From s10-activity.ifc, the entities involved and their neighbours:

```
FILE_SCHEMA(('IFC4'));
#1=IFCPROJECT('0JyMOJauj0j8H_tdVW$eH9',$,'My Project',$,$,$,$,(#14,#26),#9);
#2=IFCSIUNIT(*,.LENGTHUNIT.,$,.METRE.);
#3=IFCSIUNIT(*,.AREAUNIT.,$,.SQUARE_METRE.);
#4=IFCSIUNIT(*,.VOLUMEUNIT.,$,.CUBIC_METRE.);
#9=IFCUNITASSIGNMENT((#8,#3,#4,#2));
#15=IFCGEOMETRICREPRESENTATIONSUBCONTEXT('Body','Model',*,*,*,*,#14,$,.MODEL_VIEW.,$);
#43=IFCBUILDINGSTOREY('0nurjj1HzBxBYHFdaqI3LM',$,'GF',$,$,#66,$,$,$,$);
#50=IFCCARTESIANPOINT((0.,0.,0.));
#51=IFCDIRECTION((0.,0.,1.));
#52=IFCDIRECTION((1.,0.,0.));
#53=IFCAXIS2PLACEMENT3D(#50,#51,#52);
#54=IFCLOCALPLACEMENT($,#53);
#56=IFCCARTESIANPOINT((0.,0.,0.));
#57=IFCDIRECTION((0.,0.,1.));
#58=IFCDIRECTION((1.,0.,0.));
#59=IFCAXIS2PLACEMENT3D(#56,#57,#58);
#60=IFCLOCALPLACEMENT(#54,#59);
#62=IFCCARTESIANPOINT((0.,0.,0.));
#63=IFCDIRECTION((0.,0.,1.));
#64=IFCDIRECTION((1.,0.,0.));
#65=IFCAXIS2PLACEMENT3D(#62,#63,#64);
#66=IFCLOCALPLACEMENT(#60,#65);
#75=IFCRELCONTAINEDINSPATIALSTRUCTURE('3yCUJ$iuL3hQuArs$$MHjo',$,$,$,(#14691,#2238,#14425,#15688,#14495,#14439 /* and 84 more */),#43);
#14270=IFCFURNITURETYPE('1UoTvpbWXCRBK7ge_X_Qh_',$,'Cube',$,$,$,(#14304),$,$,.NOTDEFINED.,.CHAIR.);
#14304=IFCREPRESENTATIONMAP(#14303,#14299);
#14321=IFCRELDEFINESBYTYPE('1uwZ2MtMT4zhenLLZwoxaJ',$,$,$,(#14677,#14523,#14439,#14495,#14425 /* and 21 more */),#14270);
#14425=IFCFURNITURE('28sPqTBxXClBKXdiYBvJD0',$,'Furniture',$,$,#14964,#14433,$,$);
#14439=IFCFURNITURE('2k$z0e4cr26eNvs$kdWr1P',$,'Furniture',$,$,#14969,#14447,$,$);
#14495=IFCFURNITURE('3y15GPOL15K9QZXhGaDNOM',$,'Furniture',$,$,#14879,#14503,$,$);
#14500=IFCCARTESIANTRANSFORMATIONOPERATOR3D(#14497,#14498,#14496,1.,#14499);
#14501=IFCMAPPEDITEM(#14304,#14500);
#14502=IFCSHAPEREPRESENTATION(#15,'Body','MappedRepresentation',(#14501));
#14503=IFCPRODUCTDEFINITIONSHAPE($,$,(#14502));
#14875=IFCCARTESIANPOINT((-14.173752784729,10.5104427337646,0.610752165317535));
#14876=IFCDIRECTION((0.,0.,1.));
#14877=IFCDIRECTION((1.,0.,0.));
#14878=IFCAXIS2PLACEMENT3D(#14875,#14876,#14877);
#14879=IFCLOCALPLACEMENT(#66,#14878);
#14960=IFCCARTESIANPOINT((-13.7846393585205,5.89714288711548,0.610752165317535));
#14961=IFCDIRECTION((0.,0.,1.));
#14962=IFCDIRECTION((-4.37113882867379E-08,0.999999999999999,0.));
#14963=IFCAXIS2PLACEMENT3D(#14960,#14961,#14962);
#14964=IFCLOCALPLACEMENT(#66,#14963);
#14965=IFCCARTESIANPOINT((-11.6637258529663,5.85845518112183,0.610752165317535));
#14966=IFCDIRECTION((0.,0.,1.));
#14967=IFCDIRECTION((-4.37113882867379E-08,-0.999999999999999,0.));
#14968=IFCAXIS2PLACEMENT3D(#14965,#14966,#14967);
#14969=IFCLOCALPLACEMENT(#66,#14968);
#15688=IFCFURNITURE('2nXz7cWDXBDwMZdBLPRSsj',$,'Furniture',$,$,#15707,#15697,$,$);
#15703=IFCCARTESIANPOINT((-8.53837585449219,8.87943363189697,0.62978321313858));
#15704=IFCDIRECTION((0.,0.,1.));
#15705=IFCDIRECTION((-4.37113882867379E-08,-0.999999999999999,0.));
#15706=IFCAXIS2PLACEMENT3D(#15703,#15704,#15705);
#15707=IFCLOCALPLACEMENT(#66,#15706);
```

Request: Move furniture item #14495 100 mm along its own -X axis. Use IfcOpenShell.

```python
import ifcopenshell
import ifcopenshell.api.geometry
import ifcopenshell.util.placement
import ifcopenshell.util.unit

model = ifcopenshell.open("s10-activity.ifc")
unit_scale = ifcopenshell.util.unit.calculate_unit_scale(model)

item = model.by_id(14495)
matrix = ifcopenshell.util.placement.get_local_placement(item.ObjectPlacement)
matrix[:3, 3] -= matrix[:3, 0] * 0.1 / unit_scale
ifcopenshell.api.geometry.edit_object_placement(model, product=item, matrix=matrix, is_si=False)

print(ifcopenshell.util.placement.get_local_placement(item.ObjectPlacement).round(3) + 0.0)

model.write("s10-activity_edited.ifc")
```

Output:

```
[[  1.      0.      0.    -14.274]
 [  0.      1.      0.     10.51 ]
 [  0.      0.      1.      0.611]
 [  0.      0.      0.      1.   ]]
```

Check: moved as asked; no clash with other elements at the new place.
